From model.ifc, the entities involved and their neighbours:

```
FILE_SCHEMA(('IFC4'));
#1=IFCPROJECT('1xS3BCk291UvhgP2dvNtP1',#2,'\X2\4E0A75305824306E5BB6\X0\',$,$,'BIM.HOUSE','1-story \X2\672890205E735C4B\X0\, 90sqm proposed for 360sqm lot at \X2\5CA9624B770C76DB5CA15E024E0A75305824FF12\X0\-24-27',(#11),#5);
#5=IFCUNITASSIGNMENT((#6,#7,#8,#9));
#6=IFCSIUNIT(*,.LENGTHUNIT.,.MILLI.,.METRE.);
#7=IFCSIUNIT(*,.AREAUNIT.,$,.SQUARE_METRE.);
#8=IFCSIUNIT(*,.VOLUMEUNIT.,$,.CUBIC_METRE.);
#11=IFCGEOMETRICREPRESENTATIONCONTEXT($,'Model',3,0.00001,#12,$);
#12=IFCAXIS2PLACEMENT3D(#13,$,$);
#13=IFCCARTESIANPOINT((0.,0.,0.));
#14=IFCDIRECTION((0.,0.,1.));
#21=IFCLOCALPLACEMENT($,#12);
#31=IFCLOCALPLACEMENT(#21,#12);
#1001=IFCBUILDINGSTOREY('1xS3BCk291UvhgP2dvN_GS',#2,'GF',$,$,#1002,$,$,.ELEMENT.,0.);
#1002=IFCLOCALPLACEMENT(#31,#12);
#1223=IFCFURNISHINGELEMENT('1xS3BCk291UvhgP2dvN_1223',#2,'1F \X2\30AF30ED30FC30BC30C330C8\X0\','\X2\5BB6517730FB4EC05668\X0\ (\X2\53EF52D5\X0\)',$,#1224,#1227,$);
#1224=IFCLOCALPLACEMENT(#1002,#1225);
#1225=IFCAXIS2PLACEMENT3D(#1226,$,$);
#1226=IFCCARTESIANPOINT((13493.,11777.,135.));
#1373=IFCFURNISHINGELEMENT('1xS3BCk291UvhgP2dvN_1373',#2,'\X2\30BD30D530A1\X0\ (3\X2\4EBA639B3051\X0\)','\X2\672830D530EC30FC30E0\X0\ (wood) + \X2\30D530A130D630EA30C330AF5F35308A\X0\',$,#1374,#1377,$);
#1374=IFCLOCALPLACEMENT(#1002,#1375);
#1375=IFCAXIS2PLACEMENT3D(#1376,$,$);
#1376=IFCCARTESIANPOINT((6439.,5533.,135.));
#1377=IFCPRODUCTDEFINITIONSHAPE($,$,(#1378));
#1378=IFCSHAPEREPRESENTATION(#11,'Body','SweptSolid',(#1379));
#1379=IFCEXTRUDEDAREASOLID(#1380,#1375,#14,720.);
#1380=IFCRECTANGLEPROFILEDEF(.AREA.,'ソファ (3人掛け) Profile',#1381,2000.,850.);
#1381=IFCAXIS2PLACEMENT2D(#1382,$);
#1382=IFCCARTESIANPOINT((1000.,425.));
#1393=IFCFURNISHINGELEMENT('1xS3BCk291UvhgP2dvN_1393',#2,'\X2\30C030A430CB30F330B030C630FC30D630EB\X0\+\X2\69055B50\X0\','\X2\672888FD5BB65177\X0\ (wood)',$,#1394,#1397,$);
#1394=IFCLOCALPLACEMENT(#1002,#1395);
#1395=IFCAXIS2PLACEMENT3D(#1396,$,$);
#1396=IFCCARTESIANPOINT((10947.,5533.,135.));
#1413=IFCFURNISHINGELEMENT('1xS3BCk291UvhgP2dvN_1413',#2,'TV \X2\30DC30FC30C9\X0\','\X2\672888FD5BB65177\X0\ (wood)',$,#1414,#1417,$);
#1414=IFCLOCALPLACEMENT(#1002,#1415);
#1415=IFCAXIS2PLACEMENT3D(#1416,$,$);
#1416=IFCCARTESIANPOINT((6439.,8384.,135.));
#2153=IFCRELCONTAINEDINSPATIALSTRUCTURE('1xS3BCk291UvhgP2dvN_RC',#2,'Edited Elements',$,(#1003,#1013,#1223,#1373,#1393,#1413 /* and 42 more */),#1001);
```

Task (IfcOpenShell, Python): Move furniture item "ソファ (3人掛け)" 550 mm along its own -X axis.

```python
import ifcopenshell
import ifcopenshell.api.geometry
import ifcopenshell.util.placement

model = ifcopenshell.open("model.ifc")

item = model.by_guid("1xS3BCk291UvhgP2dvN_1373")
matrix = ifcopenshell.util.placement.get_local_placement(item.ObjectPlacement)
matrix[:3, 3] -= matrix[:3, 0] * 550.0
ifcopenshell.api.geometry.edit_object_placement(model, product=item, matrix=matrix, is_si=False)

print(ifcopenshell.util.placement.get_local_placement(item.ObjectPlacement).round(3) + 0.0)

model.write("model_v2.ifc")
```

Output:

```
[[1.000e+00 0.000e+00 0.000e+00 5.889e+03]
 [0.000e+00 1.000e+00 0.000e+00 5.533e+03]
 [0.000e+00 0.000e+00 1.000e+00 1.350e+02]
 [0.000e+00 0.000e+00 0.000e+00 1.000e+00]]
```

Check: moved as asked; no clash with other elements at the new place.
